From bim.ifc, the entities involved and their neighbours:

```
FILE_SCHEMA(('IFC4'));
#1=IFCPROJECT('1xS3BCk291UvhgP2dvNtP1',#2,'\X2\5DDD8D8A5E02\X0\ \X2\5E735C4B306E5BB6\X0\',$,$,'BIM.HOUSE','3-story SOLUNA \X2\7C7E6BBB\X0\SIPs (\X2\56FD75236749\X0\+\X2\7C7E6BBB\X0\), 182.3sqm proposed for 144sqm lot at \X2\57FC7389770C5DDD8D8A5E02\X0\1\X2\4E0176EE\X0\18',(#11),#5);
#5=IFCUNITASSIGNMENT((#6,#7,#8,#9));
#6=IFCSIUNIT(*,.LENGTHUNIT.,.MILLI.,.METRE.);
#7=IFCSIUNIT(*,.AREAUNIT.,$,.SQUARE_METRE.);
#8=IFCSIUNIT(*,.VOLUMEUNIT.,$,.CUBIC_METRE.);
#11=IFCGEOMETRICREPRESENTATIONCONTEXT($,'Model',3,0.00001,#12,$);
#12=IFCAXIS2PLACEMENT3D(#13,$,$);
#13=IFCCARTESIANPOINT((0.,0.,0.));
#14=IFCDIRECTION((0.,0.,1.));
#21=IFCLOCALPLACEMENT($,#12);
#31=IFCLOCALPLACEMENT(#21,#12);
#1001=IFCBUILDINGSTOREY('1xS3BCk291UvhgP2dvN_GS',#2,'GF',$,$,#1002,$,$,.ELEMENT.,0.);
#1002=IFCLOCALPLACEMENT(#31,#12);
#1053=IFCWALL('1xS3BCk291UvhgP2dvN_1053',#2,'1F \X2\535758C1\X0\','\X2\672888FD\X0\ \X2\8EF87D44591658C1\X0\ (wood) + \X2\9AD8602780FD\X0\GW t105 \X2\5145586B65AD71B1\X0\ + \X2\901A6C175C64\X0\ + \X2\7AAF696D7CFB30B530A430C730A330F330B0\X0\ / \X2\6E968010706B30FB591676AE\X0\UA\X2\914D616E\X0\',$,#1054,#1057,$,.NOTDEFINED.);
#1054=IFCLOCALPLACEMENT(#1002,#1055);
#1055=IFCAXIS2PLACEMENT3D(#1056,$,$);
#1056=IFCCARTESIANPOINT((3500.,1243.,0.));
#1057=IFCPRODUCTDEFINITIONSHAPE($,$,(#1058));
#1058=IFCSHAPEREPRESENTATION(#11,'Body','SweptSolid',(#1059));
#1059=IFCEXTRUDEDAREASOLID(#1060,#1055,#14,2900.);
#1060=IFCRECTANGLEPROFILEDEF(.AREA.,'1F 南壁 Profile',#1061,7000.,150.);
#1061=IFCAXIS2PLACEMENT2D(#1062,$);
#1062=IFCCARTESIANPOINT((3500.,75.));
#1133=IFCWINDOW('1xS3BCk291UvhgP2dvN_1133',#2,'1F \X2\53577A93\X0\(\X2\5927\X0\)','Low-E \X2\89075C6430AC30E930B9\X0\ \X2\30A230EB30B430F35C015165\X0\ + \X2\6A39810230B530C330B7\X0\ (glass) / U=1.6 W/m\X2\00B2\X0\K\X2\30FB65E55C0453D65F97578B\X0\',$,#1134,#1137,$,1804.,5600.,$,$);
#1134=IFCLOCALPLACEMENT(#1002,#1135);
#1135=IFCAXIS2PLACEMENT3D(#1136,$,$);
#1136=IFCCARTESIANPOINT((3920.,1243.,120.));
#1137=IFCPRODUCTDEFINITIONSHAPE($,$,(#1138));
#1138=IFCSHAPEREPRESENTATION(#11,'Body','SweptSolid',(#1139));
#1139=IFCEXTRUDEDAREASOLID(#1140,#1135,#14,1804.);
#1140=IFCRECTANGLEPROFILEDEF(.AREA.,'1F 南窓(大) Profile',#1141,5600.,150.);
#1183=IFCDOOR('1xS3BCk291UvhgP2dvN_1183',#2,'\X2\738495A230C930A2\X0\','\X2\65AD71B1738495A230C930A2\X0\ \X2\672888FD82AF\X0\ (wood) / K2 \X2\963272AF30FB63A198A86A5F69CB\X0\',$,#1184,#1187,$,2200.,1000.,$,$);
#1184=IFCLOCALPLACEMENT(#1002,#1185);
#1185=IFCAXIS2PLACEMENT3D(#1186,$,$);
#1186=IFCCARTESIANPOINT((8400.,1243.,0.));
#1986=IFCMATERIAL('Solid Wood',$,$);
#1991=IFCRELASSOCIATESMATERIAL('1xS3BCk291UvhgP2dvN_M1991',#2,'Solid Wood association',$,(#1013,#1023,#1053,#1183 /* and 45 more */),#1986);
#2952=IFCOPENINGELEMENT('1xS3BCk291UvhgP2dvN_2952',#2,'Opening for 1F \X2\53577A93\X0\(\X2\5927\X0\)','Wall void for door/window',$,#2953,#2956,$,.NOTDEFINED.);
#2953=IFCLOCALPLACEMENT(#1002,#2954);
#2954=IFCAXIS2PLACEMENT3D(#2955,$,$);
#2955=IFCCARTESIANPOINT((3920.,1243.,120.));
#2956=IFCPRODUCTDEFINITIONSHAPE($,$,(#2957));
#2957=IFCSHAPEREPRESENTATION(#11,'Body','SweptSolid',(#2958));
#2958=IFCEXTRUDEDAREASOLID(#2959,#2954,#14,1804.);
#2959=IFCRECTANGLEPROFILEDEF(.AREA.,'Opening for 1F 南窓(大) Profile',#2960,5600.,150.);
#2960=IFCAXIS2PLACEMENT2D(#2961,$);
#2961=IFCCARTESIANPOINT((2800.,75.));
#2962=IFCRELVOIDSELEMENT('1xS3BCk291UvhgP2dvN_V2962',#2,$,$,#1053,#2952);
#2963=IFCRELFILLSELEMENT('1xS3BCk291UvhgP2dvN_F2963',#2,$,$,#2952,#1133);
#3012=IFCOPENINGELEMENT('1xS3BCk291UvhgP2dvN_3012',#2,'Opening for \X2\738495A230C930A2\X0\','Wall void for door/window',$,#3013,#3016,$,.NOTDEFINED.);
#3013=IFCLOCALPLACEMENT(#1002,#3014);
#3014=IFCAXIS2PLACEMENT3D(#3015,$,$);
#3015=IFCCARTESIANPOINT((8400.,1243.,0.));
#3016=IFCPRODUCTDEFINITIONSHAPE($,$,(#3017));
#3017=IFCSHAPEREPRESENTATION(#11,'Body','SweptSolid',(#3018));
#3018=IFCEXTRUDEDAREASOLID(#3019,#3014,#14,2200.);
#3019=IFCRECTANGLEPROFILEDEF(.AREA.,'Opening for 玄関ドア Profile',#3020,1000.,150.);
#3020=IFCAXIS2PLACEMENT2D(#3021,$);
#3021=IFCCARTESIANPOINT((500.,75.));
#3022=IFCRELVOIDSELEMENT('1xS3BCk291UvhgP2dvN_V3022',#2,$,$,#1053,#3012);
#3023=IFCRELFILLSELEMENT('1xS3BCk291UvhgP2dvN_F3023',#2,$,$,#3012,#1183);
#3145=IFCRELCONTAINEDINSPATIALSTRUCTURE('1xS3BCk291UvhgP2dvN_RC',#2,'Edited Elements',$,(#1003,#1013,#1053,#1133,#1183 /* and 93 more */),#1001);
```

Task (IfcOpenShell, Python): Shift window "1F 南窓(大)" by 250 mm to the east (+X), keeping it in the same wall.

```python
import ifcopenshell
import ifcopenshell.api.geometry
import ifcopenshell.util.placement
import ifcopenshell.util.unit

model = ifcopenshell.open("bim.ifc")
unit_scale = ifcopenshell.util.unit.calculate_unit_scale(model)

window = model.by_guid("1xS3BCk291UvhgP2dvN_1133")
opening = window.FillsVoids[0].RelatingOpeningElement
wall = opening.VoidsElements[0].RelatingBuildingElement

wall_matrix = ifcopenshell.util.placement.get_local_placement(wall.ObjectPlacement)
shift = wall_matrix[:3, 0] * 0.25 / unit_scale
before = ifcopenshell.util.placement.get_local_placement(window.ObjectPlacement)[:3, 3].copy()

# The window is not placed relative to its opening, so move both.
for product in (opening, window):
    matrix = ifcopenshell.util.placement.get_local_placement(product.ObjectPlacement)
    matrix[:3, 3] += shift
    ifcopenshell.api.geometry.edit_object_placement(model, product=product, matrix=matrix, is_si=False)

after = ifcopenshell.util.placement.get_local_placement(window.ObjectPlacement)[:3, 3]
print("window moved by", (after - before).round(3) + 0.0)

model.write("bim_updated.ifc")
```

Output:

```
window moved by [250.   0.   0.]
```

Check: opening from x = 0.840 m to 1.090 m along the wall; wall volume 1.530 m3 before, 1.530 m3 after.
